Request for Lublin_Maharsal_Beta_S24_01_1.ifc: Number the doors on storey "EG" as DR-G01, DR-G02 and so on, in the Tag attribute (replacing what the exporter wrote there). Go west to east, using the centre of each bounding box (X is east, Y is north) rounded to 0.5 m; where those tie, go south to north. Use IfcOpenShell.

First a look at what the model holds.

```python
import ifcopenshell
import ifcopenshell.util.element
import ifcopenshell.util.placement

model = ifcopenshell.open("Lublin_Maharsal_Beta_S24_01_1.ifc")
print(model.schema)
storey = next(s for s in model.by_type("IfcBuildingStorey") if s.Name == "EG")
doors = [e for e in ifcopenshell.util.element.get_decomposition(storey) if e.is_a("IfcDoor")]
for e in sorted(doors, key=lambda e: e.id()):
    origin = ifcopenshell.util.placement.get_local_placement(e.ObjectPlacement)[:3, 3]
    print(e.id(), e.Tag, e.Name, origin.round(2) + 0.0, sep=" | ")
```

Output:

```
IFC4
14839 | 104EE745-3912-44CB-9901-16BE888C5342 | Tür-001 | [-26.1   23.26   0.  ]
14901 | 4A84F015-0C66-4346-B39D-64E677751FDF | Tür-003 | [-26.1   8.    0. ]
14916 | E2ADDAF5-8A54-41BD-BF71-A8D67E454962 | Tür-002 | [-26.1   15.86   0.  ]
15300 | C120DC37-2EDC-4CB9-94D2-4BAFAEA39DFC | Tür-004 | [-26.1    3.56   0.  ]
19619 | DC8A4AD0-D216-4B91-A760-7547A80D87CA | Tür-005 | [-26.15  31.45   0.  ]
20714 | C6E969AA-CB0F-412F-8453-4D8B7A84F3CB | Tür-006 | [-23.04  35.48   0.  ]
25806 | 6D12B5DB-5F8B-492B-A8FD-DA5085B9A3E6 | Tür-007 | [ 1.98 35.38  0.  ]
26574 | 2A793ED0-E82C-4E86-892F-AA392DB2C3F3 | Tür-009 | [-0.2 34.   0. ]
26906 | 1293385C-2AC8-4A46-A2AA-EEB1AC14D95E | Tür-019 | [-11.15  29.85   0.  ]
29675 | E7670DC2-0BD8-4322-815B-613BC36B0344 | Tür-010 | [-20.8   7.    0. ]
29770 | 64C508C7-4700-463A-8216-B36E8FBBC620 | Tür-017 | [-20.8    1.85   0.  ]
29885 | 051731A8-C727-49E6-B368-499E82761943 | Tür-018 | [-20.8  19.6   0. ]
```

```python
import ifcopenshell
import ifcopenshell.geom
import ifcopenshell.util.element
import ifcopenshell.util.shape

model = ifcopenshell.open("Lublin_Maharsal_Beta_S24_01_1.ifc")
settings = ifcopenshell.geom.settings()
settings.set("use-world-coords", True)


def centre(element):
    shape = ifcopenshell.geom.create_shape(settings, element)
    return ifcopenshell.util.shape.get_bbox_centroid(shape.geometry)


storey = next(s for s in model.by_type("IfcBuildingStorey") if s.Name == "EG")
doors = [e for e in ifcopenshell.util.element.get_decomposition(storey) if e.is_a("IfcDoor")]

# Insertion points can sit at a corner or the storey origin, so sort by the geometry (in metres).
centres = {e: centre(e) for e in doors}
doors.sort(key=lambda e: (round(centres[e][0] / 0.5), centres[e][1]))

for i, e in enumerate(doors, start=1):
    number = f"DR-G{i:02d}"
    e.Tag = number
    print(e.id(), number)

model.write("Lublin_Maharsal_Beta_S24_01_1_edited.ifc")
```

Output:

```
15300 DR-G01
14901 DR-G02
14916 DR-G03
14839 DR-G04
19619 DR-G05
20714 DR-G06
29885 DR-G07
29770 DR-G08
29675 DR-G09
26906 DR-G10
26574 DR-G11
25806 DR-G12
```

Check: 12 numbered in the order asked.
